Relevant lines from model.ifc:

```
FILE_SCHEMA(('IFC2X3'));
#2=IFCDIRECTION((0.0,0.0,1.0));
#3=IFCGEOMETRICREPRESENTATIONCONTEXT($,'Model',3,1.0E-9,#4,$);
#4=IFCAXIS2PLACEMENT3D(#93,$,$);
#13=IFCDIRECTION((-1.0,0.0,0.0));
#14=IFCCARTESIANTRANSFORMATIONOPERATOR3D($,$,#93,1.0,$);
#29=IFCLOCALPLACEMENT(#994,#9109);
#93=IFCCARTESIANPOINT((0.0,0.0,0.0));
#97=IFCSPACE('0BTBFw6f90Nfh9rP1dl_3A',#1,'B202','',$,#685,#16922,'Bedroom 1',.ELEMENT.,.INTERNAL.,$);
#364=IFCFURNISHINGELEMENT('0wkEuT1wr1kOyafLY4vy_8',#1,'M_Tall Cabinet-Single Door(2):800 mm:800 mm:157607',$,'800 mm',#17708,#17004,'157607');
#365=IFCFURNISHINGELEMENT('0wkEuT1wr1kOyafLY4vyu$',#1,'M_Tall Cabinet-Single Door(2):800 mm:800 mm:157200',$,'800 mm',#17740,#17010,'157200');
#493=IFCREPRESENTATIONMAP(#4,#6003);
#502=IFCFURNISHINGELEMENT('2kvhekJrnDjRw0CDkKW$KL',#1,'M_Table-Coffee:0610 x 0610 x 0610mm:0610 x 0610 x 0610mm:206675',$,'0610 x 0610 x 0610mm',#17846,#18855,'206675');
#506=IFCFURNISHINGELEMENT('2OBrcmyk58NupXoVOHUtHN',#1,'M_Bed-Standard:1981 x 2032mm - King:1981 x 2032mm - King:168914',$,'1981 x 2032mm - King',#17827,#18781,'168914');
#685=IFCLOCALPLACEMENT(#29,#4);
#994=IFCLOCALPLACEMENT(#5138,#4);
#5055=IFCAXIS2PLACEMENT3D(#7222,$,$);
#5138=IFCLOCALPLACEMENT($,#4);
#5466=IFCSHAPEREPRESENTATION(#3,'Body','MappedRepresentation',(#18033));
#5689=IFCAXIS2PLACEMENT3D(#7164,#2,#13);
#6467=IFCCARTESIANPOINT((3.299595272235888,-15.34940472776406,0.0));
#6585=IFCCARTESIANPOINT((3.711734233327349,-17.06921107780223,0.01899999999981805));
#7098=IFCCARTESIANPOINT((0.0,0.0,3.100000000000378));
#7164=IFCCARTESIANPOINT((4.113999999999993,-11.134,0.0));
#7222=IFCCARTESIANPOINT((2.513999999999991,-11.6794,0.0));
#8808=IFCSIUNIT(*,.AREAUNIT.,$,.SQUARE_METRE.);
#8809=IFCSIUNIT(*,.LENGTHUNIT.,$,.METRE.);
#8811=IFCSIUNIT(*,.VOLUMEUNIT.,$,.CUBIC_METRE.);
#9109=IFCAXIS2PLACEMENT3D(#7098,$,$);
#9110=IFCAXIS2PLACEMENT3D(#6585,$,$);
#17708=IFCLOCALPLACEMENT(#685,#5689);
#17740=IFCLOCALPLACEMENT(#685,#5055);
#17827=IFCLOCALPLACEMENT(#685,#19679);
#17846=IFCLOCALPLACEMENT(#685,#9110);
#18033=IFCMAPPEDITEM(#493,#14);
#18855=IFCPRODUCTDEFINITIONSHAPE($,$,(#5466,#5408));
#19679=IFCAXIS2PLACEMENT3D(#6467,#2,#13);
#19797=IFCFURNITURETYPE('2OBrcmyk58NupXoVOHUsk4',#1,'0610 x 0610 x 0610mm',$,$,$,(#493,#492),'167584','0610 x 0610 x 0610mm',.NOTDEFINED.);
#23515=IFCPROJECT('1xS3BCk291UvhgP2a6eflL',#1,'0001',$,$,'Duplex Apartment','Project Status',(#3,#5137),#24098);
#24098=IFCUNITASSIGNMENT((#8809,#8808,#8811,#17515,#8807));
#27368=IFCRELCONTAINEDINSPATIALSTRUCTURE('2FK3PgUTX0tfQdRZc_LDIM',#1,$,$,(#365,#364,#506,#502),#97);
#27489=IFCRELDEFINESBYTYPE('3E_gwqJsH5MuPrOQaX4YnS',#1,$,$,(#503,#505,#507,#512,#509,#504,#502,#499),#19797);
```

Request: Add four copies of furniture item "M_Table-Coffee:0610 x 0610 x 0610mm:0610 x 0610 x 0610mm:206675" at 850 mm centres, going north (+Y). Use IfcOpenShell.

```python
import numpy as np
import ifcopenshell
import ifcopenshell.api.geometry
import ifcopenshell.api.root
import ifcopenshell.util.element
import ifcopenshell.util.placement
import ifcopenshell.util.unit

model = ifcopenshell.open("model.ifc")
unit_scale = ifcopenshell.util.unit.calculate_unit_scale(model)


def reuse_history(source, copy):
    """copy_class also copies each property set's owner history, people and application; keep the originals."""
    for rel in copy.IsDefinedBy:
        if rel.is_a("IfcRelDefinesByProperties") and (history := rel.RelatingPropertyDefinition.OwnerHistory):
            rel.RelatingPropertyDefinition.OwnerHistory = source.OwnerHistory
            ifcopenshell.util.element.remove_deep2(model, history)


source = model.by_guid("2kvhekJrnDjRw0CDkKW$KL")
base = ifcopenshell.util.placement.get_local_placement(source.ObjectPlacement)
step = np.array([0.0, 1.0, 0.0]) * 0.85 / unit_scale

for i in range(1, 5):
    copy = ifcopenshell.api.root.copy_class(model, product=source)
    copy.Representation = ifcopenshell.util.element.copy_deep(
        model, source.Representation, exclude=["IfcGeometricRepresentationContext", "IfcRepresentationMap"]
    )
    copy.Name = "M_Table-Coffee:0610 x 0610 x 0610mm:0610 x 0610 x 0610mm"
    copy.Tag = None
    reuse_history(source, copy)
    matrix = base.copy()
    matrix[:3, 3] += i * step
    print("added at", matrix[:3, 3].round(3) + 0.0)
    ifcopenshell.api.geometry.edit_object_placement(model, product=copy, matrix=matrix, is_si=False)

model.write("model_rev.ifc")
```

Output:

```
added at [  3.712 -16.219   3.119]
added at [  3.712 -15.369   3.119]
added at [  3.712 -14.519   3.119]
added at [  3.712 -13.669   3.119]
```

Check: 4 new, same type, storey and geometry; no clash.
